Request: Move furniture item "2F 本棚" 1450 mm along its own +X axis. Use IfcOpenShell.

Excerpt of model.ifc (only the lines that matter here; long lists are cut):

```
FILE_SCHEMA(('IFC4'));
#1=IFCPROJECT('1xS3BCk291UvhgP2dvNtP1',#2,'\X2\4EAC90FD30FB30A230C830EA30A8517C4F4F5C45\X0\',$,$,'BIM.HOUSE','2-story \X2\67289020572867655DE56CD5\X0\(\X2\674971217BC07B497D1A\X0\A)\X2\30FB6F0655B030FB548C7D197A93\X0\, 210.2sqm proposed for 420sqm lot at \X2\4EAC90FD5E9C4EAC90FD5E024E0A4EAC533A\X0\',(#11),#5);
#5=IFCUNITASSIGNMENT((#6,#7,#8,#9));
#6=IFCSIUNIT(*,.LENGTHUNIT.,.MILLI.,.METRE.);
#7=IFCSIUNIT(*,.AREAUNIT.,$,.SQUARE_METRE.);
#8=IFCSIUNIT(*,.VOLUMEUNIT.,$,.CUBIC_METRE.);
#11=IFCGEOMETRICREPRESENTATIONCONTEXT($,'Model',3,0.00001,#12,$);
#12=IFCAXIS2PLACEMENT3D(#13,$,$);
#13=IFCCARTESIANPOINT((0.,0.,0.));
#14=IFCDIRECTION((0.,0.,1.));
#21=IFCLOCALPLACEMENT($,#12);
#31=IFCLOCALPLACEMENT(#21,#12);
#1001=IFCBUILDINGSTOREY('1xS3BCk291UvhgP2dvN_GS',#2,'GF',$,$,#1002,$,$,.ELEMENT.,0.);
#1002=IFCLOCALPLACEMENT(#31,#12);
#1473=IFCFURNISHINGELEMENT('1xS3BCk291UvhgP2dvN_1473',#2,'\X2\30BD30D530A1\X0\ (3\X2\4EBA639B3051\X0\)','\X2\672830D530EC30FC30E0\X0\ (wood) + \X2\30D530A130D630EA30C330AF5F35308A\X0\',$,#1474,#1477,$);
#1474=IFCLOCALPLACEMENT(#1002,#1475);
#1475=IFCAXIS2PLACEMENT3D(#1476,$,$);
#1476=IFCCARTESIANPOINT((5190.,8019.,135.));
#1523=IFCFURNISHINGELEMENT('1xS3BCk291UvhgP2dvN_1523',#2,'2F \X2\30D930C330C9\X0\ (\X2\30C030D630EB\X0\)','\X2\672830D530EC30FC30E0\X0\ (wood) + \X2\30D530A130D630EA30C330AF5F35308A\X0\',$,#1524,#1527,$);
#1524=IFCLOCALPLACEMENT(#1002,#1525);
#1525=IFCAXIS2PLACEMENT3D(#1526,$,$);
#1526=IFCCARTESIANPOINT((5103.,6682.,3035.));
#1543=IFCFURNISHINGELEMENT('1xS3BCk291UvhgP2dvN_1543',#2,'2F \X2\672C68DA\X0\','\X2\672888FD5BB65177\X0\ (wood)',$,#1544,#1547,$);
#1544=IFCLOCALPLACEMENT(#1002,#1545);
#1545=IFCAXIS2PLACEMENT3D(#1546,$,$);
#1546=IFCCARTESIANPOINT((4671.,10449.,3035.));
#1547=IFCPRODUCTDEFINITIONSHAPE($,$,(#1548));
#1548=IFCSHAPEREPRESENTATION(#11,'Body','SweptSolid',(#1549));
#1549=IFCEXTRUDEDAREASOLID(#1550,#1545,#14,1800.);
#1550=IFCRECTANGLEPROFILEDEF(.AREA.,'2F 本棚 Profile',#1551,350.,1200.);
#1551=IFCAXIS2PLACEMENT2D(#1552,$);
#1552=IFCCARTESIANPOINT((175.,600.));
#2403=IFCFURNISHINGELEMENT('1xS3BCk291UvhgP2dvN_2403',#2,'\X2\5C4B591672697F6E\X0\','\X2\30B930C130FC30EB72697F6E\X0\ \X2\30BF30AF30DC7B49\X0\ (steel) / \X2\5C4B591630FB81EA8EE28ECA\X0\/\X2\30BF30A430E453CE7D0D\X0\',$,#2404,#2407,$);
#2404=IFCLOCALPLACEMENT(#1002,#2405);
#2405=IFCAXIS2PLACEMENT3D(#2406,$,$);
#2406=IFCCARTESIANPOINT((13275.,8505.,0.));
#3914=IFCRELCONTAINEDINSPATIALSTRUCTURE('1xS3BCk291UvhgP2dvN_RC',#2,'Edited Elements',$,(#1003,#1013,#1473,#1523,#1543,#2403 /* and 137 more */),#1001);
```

```python
import ifcopenshell
import ifcopenshell.api.geometry
import ifcopenshell.util.placement

model = ifcopenshell.open("model.ifc")

item = model.by_guid("1xS3BCk291UvhgP2dvN_1543")
matrix = ifcopenshell.util.placement.get_local_placement(item.ObjectPlacement)
matrix[:3, 3] += matrix[:3, 0] * 1450.0
ifcopenshell.api.geometry.edit_object_placement(model, product=item, matrix=matrix, is_si=False)

print(ifcopenshell.util.placement.get_local_placement(item.ObjectPlacement).round(3) + 0.0)

model.write("model_edited.ifc")
```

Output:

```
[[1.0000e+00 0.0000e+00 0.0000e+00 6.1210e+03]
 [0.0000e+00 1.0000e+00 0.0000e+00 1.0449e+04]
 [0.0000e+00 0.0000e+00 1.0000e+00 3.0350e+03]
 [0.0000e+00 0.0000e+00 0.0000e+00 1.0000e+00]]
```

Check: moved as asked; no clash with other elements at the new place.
